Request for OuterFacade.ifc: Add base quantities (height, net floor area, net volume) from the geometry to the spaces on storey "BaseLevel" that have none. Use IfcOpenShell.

First a look at what the model holds.

```python
import ifcopenshell
import ifcopenshell.util.element
import ifcopenshell.util.unit

model = ifcopenshell.open("OuterFacade.ifc")
print(model.schema)
for unit_type in ("LENGTHUNIT", "AREAUNIT", "VOLUMEUNIT"):
    print(unit_type, ifcopenshell.util.unit.calculate_unit_scale(model, unit_type))
storey = next(s for s in model.by_type("IfcBuildingStorey") if s.Name == "BaseLevel")
spaces = [e for e in ifcopenshell.util.element.get_decomposition(storey) if e.is_a("IfcSpace")]
for e in sorted(spaces, key=lambda e: e.id()):
    print(e.id(), e.is_a(), e.Name, list(ifcopenshell.util.element.get_psets(e, qtos_only=True)), sep=" | ")
```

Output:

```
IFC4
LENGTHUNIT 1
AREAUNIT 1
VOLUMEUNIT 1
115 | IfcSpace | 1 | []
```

```python
import ifcopenshell
import ifcopenshell.api.pset
import ifcopenshell.geom
import ifcopenshell.util.element
import ifcopenshell.util.shape
import ifcopenshell.util.unit

model = ifcopenshell.open("OuterFacade.ifc")
unit_scale = ifcopenshell.util.unit.calculate_unit_scale(model)
area_scale = ifcopenshell.util.unit.calculate_unit_scale(model, "AREAUNIT")
volume_scale = ifcopenshell.util.unit.calculate_unit_scale(model, "VOLUMEUNIT")
settings = ifcopenshell.geom.settings()

storey = next(s for s in model.by_type("IfcBuildingStorey") if s.Name == "BaseLevel")
spaces = [e for e in ifcopenshell.util.element.get_decomposition(storey) if e.is_a("IfcSpace")]

for e in sorted(spaces, key=lambda e: e.id()):
    if ifcopenshell.util.element.get_psets(e, qtos_only=True, should_inherit=False):
        continue
    # Geometry comes back in metres, in the element's own axes.
    shape = ifcopenshell.geom.create_shape(settings, e)
    values = {
        "Height": ifcopenshell.util.shape.get_z(shape.geometry) / unit_scale,
        "NetFloorArea": ifcopenshell.util.shape.get_footprint_area(shape.geometry) / area_scale,
        "NetVolume": ifcopenshell.util.shape.get_volume(shape.geometry) / volume_scale,
    }
    qto = ifcopenshell.api.pset.add_qto(model, product=e, name="Qto_SpaceBaseQuantities")
    ifcopenshell.api.pset.edit_qto(model, qto=qto, properties=values)
    print(e.id(), {k: round(v, 3) for k, v in values.items()})

model.write("OuterFacade_rev.ifc")
```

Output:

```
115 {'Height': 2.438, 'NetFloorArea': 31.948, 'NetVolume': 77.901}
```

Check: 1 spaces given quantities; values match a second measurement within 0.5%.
